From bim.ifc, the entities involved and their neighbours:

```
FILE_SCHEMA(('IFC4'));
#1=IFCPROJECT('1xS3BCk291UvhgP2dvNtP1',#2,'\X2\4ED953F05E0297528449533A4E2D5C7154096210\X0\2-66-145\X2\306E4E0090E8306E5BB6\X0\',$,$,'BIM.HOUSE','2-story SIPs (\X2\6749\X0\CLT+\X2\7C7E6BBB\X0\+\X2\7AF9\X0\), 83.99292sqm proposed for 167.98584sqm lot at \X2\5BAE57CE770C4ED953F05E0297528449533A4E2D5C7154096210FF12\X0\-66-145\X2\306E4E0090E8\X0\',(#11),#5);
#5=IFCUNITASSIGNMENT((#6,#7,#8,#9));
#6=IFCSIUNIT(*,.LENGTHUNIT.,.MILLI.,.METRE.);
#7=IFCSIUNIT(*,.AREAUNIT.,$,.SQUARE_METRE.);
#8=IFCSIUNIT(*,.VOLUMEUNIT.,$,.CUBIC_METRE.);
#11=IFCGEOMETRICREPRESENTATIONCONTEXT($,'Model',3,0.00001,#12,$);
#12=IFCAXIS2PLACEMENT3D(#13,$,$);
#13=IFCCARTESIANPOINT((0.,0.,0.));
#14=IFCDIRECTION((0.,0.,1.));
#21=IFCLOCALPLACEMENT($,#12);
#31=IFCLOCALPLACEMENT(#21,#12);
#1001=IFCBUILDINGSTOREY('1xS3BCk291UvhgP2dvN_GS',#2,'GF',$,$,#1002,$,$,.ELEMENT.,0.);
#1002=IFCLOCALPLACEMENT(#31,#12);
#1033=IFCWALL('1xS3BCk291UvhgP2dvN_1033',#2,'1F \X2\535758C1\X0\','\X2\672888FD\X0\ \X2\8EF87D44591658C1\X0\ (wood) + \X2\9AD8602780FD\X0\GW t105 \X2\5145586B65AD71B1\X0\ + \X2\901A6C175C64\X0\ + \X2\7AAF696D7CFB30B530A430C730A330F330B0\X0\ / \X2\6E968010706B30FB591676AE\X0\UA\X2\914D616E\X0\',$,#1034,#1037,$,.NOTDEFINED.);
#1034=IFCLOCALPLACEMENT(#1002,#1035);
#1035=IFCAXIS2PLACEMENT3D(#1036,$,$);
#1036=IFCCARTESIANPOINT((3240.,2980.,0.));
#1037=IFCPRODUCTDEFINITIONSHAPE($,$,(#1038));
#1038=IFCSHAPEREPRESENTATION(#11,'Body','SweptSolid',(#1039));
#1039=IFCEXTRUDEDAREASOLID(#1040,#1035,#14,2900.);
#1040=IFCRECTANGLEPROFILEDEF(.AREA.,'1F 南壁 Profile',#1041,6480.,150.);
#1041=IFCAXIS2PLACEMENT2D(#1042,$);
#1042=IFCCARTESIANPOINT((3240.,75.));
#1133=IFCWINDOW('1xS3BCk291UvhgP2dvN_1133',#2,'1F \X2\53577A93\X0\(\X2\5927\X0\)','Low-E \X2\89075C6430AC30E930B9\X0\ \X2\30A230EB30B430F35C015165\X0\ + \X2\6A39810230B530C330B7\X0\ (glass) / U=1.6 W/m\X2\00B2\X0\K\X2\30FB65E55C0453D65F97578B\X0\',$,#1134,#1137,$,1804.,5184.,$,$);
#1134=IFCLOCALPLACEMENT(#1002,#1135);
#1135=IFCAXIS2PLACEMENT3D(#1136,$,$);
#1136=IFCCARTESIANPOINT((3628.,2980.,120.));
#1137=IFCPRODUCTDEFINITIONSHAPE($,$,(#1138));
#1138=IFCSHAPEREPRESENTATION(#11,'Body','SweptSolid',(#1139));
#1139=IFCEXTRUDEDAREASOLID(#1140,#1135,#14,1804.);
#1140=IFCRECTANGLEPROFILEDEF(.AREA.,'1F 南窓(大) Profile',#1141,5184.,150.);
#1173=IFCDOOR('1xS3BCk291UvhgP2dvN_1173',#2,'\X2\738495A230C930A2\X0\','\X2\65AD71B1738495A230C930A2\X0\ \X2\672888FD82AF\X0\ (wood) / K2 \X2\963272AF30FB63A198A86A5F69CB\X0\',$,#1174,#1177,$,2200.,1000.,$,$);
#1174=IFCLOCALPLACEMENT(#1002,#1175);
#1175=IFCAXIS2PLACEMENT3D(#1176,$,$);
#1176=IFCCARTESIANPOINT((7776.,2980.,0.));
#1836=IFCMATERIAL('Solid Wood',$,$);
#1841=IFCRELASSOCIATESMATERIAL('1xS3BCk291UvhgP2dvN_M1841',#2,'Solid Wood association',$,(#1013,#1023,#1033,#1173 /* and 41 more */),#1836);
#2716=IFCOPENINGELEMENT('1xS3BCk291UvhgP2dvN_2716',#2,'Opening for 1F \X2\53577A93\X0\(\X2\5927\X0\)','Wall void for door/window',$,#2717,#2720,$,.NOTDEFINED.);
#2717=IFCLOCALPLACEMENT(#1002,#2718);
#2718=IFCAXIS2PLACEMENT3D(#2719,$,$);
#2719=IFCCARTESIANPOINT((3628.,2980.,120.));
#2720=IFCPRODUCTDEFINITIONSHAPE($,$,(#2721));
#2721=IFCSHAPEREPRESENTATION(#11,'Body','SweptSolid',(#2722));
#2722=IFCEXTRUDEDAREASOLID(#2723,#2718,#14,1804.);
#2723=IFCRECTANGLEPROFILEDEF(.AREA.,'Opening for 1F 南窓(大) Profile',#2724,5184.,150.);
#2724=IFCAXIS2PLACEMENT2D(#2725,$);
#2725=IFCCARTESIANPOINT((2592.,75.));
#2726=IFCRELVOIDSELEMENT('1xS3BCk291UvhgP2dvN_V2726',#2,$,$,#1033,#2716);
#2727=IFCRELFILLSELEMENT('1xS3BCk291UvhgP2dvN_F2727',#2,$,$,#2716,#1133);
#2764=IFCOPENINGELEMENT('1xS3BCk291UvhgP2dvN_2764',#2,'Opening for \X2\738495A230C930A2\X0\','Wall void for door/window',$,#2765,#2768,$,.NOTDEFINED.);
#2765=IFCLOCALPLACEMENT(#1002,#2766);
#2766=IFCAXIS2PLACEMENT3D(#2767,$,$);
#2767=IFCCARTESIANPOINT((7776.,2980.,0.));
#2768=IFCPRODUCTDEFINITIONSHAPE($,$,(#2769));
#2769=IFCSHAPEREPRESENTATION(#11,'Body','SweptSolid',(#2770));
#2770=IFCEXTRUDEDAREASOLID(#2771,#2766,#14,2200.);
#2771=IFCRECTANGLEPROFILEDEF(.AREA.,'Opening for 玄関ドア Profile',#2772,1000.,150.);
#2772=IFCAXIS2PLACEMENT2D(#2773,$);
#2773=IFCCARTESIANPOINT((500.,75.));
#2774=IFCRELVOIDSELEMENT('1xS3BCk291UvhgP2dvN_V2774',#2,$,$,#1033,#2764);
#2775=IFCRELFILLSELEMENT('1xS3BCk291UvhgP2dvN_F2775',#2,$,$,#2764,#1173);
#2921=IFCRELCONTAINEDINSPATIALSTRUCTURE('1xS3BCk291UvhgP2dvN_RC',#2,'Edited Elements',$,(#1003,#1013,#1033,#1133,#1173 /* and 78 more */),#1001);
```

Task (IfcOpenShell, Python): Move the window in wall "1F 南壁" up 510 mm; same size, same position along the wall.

```python
import numpy as np
import ifcopenshell
import ifcopenshell.api.geometry
import ifcopenshell.util.placement
import ifcopenshell.util.unit

model = ifcopenshell.open("bim.ifc")
unit_scale = ifcopenshell.util.unit.calculate_unit_scale(model)

window = model.by_guid("1xS3BCk291UvhgP2dvN_1133")
opening = window.FillsVoids[0].RelatingOpeningElement
dz = 0.51 / unit_scale

shift = np.array([0.0, 0.0, dz])
# The window is not placed relative to its opening, so move both.
for product in (opening, window):
    matrix = ifcopenshell.util.placement.get_local_placement(product.ObjectPlacement)
    matrix[:3, 3] += shift
    ifcopenshell.api.geometry.edit_object_placement(model, product=product, matrix=matrix, is_si=False)

print(f"moved by {dz * unit_scale:+.3f} m")

model.write("bim-out.ifc")
```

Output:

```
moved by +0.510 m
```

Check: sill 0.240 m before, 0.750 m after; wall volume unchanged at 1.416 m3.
